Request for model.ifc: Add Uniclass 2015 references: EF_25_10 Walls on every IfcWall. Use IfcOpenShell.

First a look at what the model holds.

```python
import ifcopenshell

model = ifcopenshell.open("model.ifc")
print(model.schema)
print("classifications:", [c.Name for c in model.by_type("IfcClassification")])
for ifc_class in ("IfcDoor", "IfcRoof", "IfcStair", "IfcWall", "IfcWindow"):
    print(ifc_class, len(model.by_type(ifc_class)))
```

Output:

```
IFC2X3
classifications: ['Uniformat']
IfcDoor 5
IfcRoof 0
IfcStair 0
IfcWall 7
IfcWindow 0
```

```python
import ifcopenshell
import ifcopenshell.api.classification

model = ifcopenshell.open("model.ifc")

# IFC2X3 requires Source and Edition and has no link from the project to the system.
system = model.create_entity("IfcClassification", Source="NBS", Edition="2015", Name="Uniclass 2015")

codes = {
    "IfcWall": ("EF_25_10", "Walls"),
}
for ifc_class, (code, name) in codes.items():
    products = model.by_type(ifc_class)
    ifcopenshell.api.classification.add_reference(
        model, products=products, classification=system, identification=code, name=name
    )
    print(code, len(products))

model.write("model_v2.ifc")
```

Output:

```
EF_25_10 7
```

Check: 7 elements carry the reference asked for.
